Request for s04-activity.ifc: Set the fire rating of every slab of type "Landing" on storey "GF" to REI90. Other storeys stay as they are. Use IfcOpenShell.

First a look at what the model holds.

```python
import ifcopenshell
import ifcopenshell.util.element

model = ifcopenshell.open("s04-activity.ifc")
print(model.schema)
storey = next(s for s in model.by_type("IfcBuildingStorey") if s.Name == "GF")
slabs = [e for e in ifcopenshell.util.element.get_decomposition(storey) if e.is_a("IfcSlab")]
seen = {}
for e in slabs:
    element_type = ifcopenshell.util.element.get_type(e)
    key = (element_type.Name if element_type != e and element_type else None, ifcopenshell.util.element.get_pset(e, "Pset_SlabCommon", "FireRating"))
    seen[key] = seen.get(key, 0) + 1
for (name, value), count in sorted(seen.items(), key=str):
    print(count, "x", name, "|", value)
```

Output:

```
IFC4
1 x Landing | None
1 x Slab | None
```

```python
import ifcopenshell
import ifcopenshell.api.pset
import ifcopenshell.util.element

model = ifcopenshell.open("s04-activity.ifc")

storey = next(s for s in model.by_type("IfcBuildingStorey") if s.Name == "GF")
slabs = [e for e in ifcopenshell.util.element.get_decomposition(storey) if e.is_a("IfcSlab")]

count = 0
for e in slabs:
    element_type = ifcopenshell.util.element.get_type(e)
    if element_type in (None, e) or element_type.Name != "Landing":
        continue
    # add_pset returns the element's existing set when there is one.
    pset = ifcopenshell.api.pset.add_pset(model, product=e, name="Pset_SlabCommon")
    ifcopenshell.api.pset.edit_pset(model, pset=pset, properties={"FireRating": "REI90"})
    count += 1

print(count, "slabs updated")

model.write("s04-activity_edited.ifc")
```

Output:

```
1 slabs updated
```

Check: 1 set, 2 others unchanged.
